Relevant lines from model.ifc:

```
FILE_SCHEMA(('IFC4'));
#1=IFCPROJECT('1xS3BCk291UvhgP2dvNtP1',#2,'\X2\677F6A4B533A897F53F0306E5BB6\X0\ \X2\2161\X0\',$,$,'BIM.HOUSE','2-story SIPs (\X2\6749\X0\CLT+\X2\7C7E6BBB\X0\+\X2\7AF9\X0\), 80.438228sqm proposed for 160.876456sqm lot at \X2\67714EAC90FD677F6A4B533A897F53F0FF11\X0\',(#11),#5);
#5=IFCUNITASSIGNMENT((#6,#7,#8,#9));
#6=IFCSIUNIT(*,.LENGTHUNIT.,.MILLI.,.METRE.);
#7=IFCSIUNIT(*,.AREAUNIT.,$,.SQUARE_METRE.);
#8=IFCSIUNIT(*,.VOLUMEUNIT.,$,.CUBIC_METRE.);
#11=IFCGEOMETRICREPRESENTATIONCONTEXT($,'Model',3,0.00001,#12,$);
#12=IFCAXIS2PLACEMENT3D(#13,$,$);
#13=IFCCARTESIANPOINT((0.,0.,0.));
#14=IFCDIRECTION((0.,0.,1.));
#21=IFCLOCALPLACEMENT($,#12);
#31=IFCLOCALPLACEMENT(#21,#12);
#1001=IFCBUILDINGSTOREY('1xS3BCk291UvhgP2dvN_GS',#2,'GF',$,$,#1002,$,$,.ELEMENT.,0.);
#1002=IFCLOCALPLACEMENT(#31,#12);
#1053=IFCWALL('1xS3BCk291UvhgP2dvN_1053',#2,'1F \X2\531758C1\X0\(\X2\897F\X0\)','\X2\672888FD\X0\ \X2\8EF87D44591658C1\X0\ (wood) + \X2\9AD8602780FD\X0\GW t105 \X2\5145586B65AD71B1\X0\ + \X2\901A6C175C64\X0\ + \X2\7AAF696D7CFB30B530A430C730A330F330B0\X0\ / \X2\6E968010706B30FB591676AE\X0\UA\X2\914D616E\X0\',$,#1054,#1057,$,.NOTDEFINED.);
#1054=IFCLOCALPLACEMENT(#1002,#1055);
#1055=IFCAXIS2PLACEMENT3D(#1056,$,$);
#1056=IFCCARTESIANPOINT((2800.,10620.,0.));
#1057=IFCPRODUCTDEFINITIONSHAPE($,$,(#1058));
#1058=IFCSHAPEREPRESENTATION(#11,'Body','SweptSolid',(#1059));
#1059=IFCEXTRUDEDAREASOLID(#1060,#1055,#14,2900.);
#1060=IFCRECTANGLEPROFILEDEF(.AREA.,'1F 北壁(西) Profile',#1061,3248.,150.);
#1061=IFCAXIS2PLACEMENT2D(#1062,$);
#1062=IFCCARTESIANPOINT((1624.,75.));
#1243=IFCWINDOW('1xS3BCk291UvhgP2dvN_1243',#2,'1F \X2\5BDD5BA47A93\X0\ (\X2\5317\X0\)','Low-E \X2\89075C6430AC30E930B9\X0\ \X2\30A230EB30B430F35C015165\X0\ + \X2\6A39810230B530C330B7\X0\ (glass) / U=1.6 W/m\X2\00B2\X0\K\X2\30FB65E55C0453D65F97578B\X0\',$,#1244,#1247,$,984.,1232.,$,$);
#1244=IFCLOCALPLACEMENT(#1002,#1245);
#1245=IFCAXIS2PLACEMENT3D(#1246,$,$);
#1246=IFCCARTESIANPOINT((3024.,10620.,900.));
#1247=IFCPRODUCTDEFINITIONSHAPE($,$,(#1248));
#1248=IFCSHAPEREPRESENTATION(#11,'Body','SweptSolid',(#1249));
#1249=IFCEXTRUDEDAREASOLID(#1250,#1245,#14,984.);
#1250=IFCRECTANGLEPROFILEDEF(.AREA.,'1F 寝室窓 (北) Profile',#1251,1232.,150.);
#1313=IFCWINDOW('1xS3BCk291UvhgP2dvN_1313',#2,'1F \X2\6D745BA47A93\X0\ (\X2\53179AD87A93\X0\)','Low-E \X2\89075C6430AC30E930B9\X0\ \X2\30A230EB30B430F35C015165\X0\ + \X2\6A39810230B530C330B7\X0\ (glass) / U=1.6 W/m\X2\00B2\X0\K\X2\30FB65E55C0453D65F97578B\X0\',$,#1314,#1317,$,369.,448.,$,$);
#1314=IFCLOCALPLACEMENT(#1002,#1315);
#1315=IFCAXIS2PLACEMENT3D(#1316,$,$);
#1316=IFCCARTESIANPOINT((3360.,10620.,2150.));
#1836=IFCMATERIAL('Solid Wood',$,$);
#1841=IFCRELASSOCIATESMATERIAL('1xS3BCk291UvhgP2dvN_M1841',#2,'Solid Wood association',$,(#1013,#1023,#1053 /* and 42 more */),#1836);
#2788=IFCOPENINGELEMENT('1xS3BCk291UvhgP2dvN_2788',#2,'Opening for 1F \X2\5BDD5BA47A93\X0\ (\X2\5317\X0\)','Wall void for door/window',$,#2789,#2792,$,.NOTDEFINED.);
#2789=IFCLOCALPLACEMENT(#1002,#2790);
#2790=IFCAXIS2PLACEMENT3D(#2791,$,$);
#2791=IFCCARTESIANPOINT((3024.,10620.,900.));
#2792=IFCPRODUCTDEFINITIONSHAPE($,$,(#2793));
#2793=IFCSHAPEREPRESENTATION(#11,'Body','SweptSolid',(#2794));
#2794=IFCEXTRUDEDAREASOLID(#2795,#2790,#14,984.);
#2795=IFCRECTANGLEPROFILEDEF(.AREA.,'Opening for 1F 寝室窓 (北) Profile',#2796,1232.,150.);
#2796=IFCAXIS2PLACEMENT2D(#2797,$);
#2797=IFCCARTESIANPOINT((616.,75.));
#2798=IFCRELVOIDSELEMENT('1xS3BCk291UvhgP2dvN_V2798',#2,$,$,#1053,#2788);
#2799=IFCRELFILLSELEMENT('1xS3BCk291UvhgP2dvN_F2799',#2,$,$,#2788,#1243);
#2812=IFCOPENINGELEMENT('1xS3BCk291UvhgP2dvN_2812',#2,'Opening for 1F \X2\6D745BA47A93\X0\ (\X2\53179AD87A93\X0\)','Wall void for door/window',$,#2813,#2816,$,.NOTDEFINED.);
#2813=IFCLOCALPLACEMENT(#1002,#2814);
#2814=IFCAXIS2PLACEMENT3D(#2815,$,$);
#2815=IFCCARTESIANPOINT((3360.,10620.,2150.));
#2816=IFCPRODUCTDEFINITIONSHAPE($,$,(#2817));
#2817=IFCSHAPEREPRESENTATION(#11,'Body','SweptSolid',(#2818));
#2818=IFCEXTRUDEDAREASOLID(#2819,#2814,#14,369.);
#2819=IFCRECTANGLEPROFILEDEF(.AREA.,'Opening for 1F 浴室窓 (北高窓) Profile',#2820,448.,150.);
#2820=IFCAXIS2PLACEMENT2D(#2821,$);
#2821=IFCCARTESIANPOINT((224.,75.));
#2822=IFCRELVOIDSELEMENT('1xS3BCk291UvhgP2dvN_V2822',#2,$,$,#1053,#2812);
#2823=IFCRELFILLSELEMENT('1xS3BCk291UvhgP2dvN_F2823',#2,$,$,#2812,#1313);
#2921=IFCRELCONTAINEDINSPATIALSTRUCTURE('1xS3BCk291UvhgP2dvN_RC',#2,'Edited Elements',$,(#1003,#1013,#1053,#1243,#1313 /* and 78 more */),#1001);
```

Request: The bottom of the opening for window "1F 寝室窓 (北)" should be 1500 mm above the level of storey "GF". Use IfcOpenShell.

```python
import numpy as np
import ifcopenshell
import ifcopenshell.api.geometry
import ifcopenshell.geom
import ifcopenshell.util.element
import ifcopenshell.util.placement
import ifcopenshell.util.shape
import ifcopenshell.util.unit

model = ifcopenshell.open("model.ifc")
unit_scale = ifcopenshell.util.unit.calculate_unit_scale(model)

window = model.by_guid("1xS3BCk291UvhgP2dvN_1243")
opening = window.FillsVoids[0].RelatingOpeningElement
storey = ifcopenshell.util.element.get_container(window, ifc_class="IfcBuildingStorey")
level = ifcopenshell.util.placement.get_local_placement(storey.ObjectPlacement)[2, 3]

# The opening's origin need not be at the sill, so measure its lowest point.
shape = ifcopenshell.geom.create_shape(ifcopenshell.geom.settings(), opening)
bottom = ifcopenshell.util.shape.get_shape_bottom_elevation(shape, shape.geometry) / unit_scale
dz = level + 1.5 / unit_scale - bottom

shift = np.array([0.0, 0.0, dz])
# The window is not placed relative to its opening, so move both.
for product in (opening, window):
    matrix = ifcopenshell.util.placement.get_local_placement(product.ObjectPlacement)
    matrix[:3, 3] += shift
    ifcopenshell.api.geometry.edit_object_placement(model, product=product, matrix=matrix, is_si=False)

print(f"moved by {dz * unit_scale:+.3f} m")

model.write("model_edited.ifc")
```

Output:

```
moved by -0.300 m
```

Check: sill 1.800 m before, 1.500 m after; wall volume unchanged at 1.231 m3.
